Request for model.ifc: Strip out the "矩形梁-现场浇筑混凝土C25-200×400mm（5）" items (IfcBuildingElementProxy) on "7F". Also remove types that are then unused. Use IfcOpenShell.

First a look at what the model holds.

```python
import ifcopenshell
import ifcopenshell.util.element

model = ifcopenshell.open("model.ifc")
print(model.schema)
storey = next(s for s in model.by_type("IfcBuildingStorey") if s.Name == "7F")
proxies = [e for e in ifcopenshell.util.element.get_decomposition(storey) if e.is_a("IfcBuildingElementProxy")]
seen = {}
for e in proxies:
    element_type = ifcopenshell.util.element.get_type(e)
    name = element_type.Name if element_type not in (None, e) else None
    seen[name] = seen.get(name, 0) + 1
for name, count in sorted(seen.items(), key=str):
    print(count, "x", name)
```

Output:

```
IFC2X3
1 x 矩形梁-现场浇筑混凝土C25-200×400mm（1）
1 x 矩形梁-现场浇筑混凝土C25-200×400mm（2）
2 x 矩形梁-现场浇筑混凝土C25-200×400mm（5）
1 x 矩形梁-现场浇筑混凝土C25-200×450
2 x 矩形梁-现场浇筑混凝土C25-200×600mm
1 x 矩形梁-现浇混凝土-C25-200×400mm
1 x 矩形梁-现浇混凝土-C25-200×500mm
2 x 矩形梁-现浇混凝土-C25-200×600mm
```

```python
import ifcopenshell
import ifcopenshell.api.root
import ifcopenshell.util.element

model = ifcopenshell.open("model.ifc")

storey = next(s for s in model.by_type("IfcBuildingStorey") if s.Name == "7F")
proxies = [e for e in ifcopenshell.util.element.get_decomposition(storey) if e.is_a("IfcBuildingElementProxy")]
targets = [e for e in proxies if (t := ifcopenshell.util.element.get_type(e)) not in (None, e) and t.Name == "矩形梁-现场浇筑混凝土C25-200×400mm（5）"]
types = {ifcopenshell.util.element.get_type(e) for e in targets} - {None, *targets}

for e in targets:
    ifcopenshell.api.root.remove_product(model, product=e)
print(len(targets), "removed")

unused = [t for t in types if not ifcopenshell.util.element.get_types(t)]
for t in unused:
    ifcopenshell.api.root.remove_product(model, product=t)
print(len(unused), "unused types removed")

model.write("model-out.ifc")
```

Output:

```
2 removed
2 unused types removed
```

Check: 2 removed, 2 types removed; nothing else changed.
